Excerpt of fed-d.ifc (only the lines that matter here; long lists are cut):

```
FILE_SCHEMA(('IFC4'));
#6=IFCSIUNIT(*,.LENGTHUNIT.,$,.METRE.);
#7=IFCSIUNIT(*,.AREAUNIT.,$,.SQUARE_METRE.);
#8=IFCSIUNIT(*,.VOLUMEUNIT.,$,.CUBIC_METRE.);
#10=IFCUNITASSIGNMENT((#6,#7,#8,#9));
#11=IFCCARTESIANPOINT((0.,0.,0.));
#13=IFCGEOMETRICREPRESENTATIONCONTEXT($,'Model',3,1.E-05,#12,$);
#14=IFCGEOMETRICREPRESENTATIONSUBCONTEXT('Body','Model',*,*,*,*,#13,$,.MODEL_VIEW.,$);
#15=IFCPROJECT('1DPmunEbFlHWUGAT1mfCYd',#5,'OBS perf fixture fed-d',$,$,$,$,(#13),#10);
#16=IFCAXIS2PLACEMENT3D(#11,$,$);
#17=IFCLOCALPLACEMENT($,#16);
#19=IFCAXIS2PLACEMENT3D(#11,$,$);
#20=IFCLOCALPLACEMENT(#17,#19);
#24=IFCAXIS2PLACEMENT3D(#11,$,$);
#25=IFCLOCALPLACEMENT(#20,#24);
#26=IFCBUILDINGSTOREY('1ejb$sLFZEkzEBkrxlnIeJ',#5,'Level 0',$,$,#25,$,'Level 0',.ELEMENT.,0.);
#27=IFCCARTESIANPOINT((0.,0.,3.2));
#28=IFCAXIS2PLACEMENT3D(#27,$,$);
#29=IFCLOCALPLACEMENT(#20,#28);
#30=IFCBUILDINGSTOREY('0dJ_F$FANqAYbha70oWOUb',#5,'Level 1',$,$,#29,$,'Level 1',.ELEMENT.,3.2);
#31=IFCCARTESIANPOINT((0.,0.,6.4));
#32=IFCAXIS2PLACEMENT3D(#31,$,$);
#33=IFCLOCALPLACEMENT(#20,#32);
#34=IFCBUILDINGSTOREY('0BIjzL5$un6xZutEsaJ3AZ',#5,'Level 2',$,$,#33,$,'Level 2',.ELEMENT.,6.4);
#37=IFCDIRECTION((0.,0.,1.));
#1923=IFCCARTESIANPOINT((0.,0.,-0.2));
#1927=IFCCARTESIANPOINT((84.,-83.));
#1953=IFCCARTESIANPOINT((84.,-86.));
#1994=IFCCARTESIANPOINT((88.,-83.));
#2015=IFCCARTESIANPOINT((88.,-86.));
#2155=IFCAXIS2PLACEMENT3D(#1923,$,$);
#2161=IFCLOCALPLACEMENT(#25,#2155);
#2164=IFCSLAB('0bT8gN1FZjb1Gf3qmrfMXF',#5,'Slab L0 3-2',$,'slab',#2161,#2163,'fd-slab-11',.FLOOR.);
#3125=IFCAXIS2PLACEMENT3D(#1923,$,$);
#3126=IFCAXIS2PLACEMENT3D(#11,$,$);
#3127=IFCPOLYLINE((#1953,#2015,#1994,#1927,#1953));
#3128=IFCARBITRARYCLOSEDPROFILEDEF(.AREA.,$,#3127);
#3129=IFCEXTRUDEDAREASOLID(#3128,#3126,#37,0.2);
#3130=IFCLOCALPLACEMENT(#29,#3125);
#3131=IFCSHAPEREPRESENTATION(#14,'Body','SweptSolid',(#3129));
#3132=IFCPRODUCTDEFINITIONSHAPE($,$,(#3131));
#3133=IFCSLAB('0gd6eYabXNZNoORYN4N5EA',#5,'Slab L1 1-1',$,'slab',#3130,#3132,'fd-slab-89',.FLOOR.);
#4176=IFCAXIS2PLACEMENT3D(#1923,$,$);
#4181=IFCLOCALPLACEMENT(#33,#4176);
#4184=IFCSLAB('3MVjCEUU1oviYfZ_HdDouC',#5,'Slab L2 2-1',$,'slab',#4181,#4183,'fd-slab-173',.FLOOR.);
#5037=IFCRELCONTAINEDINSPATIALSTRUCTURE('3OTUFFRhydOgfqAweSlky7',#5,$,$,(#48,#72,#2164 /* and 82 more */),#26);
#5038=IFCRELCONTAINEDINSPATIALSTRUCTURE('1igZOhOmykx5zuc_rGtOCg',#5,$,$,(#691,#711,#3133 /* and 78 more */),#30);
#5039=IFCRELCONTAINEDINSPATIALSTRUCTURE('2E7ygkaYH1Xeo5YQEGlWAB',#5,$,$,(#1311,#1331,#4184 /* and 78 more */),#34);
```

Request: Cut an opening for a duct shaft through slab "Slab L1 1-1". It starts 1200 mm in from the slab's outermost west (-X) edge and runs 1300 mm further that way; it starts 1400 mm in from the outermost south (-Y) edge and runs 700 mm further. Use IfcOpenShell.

```python
import numpy as np
import ifcopenshell
import ifcopenshell.api.feature
import ifcopenshell.api.geometry
import ifcopenshell.api.root
import ifcopenshell.geom
import ifcopenshell.util.placement
import ifcopenshell.util.representation
import ifcopenshell.util.shape
import ifcopenshell.util.unit

model = ifcopenshell.open("fed-d.ifc")
unit_scale = ifcopenshell.util.unit.calculate_unit_scale(model)
settings = ifcopenshell.geom.settings()


def volume(element):
    """Net volume in cubic metres, openings subtracted."""
    shape = ifcopenshell.geom.create_shape(settings, element)
    return ifcopenshell.util.shape.get_volume(shape.geometry)


slab = model.by_guid("0gd6eYabXNZNoORYN4N5EA")
before = volume(slab)

# Extent in the slab's own axes, in metres. The edges named are its -X and -Y sides.
slab_shape = ifcopenshell.geom.create_shape(settings, slab)
vertices = ifcopenshell.util.shape.get_vertices(slab_shape.geometry)
x_min, y_min, bottom = vertices.min(axis=0)
top = vertices[:, 2].max()

opening = ifcopenshell.api.root.create_entity(model, ifc_class="IfcOpeningElement", name="Duct shaft opening", predefined_type="OPENING")
context = ifcopenshell.util.representation.get_context(model, "Model", "Body", "MODEL_VIEW")
width, depth = 1.3, 0.7
outline = [(0.0, 0.0), (width, 0.0), (width, depth), (0.0, depth), (0.0, 0.0)]
# Overshoot both faces by 50 mm so the cut is clean.
shape = ifcopenshell.api.geometry.add_slab_representation(
    model, context=context, depth=top - bottom + 0.1, polyline=outline
)
ifcopenshell.api.geometry.assign_representation(model, product=opening, representation=shape)

matrix = ifcopenshell.util.placement.get_local_placement(slab.ObjectPlacement)
matrix[:, 3] = matrix @ np.append(np.array([x_min + 1.2, y_min + 1.4, bottom - 0.05]) / unit_scale, 1.0)
ifcopenshell.api.geometry.edit_object_placement(model, product=opening, matrix=matrix, is_si=False)
ifcopenshell.api.feature.add_feature(model, feature=opening, element=slab)

after = volume(slab)

print(f"slab volume {before:.3f} -> {after:.3f} m3")

model.write("fed-d_updated.ifc")
```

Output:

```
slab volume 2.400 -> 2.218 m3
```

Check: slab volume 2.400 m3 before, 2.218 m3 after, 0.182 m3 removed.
